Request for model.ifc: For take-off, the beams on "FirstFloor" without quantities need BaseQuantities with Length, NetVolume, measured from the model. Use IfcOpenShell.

First a look at what the model holds.

```python
import ifcopenshell
import ifcopenshell.util.element
import ifcopenshell.util.unit

model = ifcopenshell.open("model.ifc")
print(model.schema)
for unit_type in ("LENGTHUNIT", "AREAUNIT", "VOLUMEUNIT"):
    print(unit_type, ifcopenshell.util.unit.calculate_unit_scale(model, unit_type))
storey = next(s for s in model.by_type("IfcBuildingStorey") if s.Name == "FirstFloor")
beams = [e for e in ifcopenshell.util.element.get_decomposition(storey) if e.is_a("IfcBeam")]
for e in sorted(beams, key=lambda e: e.id()):
    print(e.id(), e.is_a(), e.Name, list(ifcopenshell.util.element.get_psets(e, qtos_only=True)), sep=" | ")
```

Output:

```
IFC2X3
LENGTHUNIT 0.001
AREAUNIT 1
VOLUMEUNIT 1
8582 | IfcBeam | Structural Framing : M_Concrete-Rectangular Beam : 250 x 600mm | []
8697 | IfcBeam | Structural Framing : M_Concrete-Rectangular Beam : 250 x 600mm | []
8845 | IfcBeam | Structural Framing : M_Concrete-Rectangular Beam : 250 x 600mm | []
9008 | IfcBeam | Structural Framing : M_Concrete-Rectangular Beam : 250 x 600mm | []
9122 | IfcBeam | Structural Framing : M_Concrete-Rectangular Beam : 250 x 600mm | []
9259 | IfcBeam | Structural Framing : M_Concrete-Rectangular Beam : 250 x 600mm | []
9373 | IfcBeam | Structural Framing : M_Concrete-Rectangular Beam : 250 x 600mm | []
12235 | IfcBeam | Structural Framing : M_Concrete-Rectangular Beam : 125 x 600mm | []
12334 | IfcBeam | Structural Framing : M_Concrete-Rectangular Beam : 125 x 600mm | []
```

```python
import ifcopenshell
import ifcopenshell.api.pset
import ifcopenshell.geom
import ifcopenshell.util.element
import ifcopenshell.util.shape
import ifcopenshell.util.unit

model = ifcopenshell.open("model.ifc")
unit_scale = ifcopenshell.util.unit.calculate_unit_scale(model)
volume_scale = ifcopenshell.util.unit.calculate_unit_scale(model, "VOLUMEUNIT")
settings = ifcopenshell.geom.settings()

storey = next(s for s in model.by_type("IfcBuildingStorey") if s.Name == "FirstFloor")
beams = [e for e in ifcopenshell.util.element.get_decomposition(storey) if e.is_a("IfcBeam")]

for e in sorted(beams, key=lambda e: e.id()):
    if ifcopenshell.util.element.get_psets(e, qtos_only=True, should_inherit=False):
        continue
    # Geometry comes back in metres, in the element's own axes.
    shape = ifcopenshell.geom.create_shape(settings, e)
    values = {
        "Length": ifcopenshell.util.shape.get_max_xyz(shape.geometry) / unit_scale,
        "NetVolume": ifcopenshell.util.shape.get_volume(shape.geometry) / volume_scale,
    }
    qto = ifcopenshell.api.pset.add_qto(model, product=e, name="BaseQuantities")
    ifcopenshell.api.pset.edit_qto(model, qto=qto, properties=values)
    print(e.id(), {k: round(v, 3) for k, v in values.items()})

model.write("model-out.ifc")
```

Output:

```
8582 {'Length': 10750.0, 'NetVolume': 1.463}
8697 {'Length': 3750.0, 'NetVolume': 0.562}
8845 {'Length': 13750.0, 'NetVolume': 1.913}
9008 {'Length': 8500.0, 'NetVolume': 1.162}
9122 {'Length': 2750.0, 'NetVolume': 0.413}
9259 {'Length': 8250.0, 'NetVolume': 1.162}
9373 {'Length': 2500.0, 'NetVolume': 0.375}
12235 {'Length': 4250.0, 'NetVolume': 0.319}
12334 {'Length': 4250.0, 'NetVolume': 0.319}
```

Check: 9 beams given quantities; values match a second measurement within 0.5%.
